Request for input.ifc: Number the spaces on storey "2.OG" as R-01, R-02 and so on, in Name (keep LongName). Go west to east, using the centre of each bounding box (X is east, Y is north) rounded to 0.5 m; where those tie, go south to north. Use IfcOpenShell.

First a look at what the model holds.

```python
import ifcopenshell
import ifcopenshell.util.element
import ifcopenshell.util.placement

model = ifcopenshell.open("input.ifc")
print(model.schema)
storey = next(s for s in model.by_type("IfcBuildingStorey") if s.Name == "2.OG")
spaces = [e for e in ifcopenshell.util.element.get_decomposition(storey) if e.is_a("IfcSpace")]
for e in sorted(spaces, key=lambda e: e.id()):
    origin = ifcopenshell.util.placement.get_local_placement(e.ObjectPlacement)[:3, 3]
    print(e.id(), e.Name, e.LongName, origin.round(2) + 0.0, sep=" | ")
```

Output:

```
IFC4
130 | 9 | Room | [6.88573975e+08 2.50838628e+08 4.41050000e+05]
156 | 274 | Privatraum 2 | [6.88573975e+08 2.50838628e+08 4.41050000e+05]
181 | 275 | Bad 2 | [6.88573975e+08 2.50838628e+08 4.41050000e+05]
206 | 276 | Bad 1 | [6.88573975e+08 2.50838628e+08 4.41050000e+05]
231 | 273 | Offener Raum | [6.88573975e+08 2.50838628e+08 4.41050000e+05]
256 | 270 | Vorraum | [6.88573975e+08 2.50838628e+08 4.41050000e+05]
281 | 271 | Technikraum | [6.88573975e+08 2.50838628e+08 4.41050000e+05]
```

```python
import ifcopenshell
import ifcopenshell.geom
import ifcopenshell.util.element
import ifcopenshell.util.shape

model = ifcopenshell.open("input.ifc")
settings = ifcopenshell.geom.settings()
settings.set("use-world-coords", True)


def centre(element):
    shape = ifcopenshell.geom.create_shape(settings, element)
    return ifcopenshell.util.shape.get_bbox_centroid(shape.geometry)


storey = next(s for s in model.by_type("IfcBuildingStorey") if s.Name == "2.OG")
spaces = [e for e in ifcopenshell.util.element.get_decomposition(storey) if e.is_a("IfcSpace")]

# Insertion points can sit at a corner or the storey origin, so sort by the geometry (in metres).
centres = {e: centre(e) for e in spaces}
spaces.sort(key=lambda e: (round(centres[e][0] / 0.5), centres[e][1]))

for i, e in enumerate(spaces, start=1):
    number = f"R-{i:02d}"
    e.Name = number
    print(e.id(), number)

model.write("input_rev.ifc")
```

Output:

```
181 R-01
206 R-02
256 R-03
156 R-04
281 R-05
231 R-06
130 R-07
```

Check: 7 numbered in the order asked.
